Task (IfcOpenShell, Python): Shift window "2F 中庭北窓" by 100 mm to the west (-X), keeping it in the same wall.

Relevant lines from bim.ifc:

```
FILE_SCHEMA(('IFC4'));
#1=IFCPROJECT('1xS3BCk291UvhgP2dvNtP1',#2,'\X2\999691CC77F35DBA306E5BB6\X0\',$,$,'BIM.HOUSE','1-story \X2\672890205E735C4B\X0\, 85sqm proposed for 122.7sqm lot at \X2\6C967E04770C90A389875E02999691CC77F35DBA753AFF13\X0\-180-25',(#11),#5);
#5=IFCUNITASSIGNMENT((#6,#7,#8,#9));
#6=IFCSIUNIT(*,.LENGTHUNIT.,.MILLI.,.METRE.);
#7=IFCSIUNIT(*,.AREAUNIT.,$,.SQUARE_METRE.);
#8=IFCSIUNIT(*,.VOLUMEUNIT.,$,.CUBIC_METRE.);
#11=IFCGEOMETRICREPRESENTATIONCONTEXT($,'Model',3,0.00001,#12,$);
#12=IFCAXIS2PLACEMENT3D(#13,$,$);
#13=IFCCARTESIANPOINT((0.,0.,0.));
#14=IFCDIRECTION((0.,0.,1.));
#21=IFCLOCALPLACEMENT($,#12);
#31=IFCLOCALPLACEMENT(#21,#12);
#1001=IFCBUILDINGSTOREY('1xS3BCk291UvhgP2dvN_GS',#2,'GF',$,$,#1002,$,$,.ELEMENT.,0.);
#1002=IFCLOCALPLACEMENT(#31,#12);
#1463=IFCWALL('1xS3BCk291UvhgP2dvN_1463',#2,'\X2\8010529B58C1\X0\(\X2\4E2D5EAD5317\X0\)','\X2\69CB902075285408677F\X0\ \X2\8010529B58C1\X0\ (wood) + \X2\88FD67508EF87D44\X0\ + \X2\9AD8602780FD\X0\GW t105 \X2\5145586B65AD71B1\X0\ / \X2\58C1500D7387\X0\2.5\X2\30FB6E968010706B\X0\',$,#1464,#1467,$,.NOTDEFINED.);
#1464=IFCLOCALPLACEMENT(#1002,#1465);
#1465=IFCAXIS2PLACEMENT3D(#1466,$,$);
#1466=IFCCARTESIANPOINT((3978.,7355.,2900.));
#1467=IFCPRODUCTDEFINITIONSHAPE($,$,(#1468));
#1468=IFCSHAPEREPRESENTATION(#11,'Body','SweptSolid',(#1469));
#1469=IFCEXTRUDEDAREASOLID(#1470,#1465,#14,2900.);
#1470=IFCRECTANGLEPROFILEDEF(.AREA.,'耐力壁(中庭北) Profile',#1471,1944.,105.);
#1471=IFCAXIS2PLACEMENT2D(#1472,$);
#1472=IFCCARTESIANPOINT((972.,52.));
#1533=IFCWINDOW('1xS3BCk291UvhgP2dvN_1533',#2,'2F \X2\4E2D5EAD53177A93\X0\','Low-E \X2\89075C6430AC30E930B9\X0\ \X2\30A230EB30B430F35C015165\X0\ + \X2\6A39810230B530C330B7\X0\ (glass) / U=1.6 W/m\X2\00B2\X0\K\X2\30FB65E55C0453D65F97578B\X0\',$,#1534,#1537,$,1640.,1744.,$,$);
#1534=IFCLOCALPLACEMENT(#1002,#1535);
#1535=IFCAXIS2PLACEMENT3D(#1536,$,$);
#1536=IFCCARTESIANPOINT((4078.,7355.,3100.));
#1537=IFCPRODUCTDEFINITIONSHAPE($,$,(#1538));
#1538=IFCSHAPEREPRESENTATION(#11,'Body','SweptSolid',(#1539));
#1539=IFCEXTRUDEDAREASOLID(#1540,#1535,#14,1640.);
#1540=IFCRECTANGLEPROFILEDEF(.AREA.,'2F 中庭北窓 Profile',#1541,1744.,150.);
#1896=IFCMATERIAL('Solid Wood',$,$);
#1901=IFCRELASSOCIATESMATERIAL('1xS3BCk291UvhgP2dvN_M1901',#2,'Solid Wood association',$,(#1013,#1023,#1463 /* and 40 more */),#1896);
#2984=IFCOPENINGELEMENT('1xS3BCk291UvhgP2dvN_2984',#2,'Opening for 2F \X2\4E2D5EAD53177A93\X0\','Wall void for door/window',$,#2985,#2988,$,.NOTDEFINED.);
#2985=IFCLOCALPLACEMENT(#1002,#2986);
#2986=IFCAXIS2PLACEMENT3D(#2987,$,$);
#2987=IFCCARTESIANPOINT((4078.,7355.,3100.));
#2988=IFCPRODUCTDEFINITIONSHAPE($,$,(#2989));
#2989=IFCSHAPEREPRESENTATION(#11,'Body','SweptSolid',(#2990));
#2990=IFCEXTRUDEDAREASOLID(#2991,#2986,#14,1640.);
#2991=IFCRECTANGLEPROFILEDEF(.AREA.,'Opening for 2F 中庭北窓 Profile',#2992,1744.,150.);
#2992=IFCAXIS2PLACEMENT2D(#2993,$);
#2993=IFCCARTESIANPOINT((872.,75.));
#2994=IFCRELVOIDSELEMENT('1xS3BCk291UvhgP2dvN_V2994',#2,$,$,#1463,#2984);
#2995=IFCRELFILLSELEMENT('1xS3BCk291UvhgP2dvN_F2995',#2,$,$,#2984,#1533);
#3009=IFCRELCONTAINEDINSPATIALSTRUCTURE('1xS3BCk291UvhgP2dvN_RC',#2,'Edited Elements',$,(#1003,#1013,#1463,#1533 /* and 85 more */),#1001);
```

```python
import ifcopenshell
import ifcopenshell.api.geometry
import ifcopenshell.util.placement

model = ifcopenshell.open("bim.ifc")

window = model.by_guid("1xS3BCk291UvhgP2dvN_1533")
opening = window.FillsVoids[0].RelatingOpeningElement
wall = opening.VoidsElements[0].RelatingBuildingElement

wall_matrix = ifcopenshell.util.placement.get_local_placement(wall.ObjectPlacement)
shift = wall_matrix[:3, 0] * -100.0
before = ifcopenshell.util.placement.get_local_placement(window.ObjectPlacement)[:3, 3].copy()

# The window is not placed relative to its opening, so move both.
for product in (opening, window):
    matrix = ifcopenshell.util.placement.get_local_placement(product.ObjectPlacement)
    matrix[:3, 3] += shift
    ifcopenshell.api.geometry.edit_object_placement(model, product=product, matrix=matrix, is_si=False)

after = ifcopenshell.util.placement.get_local_placement(window.ObjectPlacement)[:3, 3]
print("window moved by", (after - before).round(3) + 0.0)

model.write("bim_updated.ifc")
```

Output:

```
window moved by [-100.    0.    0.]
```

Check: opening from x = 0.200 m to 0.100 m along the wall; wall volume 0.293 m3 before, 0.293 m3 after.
